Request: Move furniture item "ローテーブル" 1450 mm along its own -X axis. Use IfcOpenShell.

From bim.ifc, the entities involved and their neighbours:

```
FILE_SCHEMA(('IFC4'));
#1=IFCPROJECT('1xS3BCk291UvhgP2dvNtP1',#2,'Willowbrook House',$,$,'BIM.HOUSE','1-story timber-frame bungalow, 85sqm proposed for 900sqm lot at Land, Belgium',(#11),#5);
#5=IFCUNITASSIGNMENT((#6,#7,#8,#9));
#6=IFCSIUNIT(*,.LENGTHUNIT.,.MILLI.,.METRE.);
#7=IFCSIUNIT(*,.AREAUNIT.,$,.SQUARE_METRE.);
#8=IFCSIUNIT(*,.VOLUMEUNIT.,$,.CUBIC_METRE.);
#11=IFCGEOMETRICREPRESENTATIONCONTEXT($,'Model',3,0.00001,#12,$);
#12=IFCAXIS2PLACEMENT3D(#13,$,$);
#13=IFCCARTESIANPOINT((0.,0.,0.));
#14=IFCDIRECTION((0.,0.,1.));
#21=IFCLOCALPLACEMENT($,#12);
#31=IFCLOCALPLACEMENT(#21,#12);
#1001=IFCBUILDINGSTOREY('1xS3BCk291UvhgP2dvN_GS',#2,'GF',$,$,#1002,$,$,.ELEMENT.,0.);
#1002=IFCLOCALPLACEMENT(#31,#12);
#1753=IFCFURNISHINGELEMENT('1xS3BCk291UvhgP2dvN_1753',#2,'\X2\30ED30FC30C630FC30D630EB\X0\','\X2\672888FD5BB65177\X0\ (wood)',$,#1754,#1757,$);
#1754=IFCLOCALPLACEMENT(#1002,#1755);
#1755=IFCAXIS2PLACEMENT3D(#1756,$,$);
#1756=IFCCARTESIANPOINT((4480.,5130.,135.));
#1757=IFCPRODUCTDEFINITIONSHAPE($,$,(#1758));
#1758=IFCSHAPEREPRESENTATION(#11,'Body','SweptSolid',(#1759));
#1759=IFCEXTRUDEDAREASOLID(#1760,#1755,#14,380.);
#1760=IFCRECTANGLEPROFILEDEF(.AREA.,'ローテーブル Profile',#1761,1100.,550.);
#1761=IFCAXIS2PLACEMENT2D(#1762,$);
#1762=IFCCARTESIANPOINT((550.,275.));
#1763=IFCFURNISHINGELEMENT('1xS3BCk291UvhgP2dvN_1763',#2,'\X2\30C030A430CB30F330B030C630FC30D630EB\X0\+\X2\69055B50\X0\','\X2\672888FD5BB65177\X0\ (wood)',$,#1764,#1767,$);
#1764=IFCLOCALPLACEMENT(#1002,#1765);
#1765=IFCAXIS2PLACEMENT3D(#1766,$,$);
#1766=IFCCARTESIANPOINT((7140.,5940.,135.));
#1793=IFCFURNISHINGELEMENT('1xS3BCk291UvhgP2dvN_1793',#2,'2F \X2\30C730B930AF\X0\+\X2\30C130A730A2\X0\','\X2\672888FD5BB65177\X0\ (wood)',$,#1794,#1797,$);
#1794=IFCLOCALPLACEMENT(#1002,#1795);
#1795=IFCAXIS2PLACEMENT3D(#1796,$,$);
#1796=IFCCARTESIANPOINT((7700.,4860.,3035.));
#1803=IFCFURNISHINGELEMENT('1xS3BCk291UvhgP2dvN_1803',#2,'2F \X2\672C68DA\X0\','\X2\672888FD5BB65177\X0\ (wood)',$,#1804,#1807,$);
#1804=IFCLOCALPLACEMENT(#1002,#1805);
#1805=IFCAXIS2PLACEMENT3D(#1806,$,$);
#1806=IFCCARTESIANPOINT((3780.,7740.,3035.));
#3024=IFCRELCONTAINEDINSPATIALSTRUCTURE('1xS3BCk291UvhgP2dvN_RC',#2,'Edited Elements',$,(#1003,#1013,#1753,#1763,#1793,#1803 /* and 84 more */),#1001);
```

```python
import ifcopenshell
import ifcopenshell.api.geometry
import ifcopenshell.util.placement
import ifcopenshell.util.unit

model = ifcopenshell.open("bim.ifc")
unit_scale = ifcopenshell.util.unit.calculate_unit_scale(model)

item = model.by_guid("1xS3BCk291UvhgP2dvN_1753")
matrix = ifcopenshell.util.placement.get_local_placement(item.ObjectPlacement)
matrix[:3, 3] -= matrix[:3, 0] * 1.45 / unit_scale
ifcopenshell.api.geometry.edit_object_placement(model, product=item, matrix=matrix, is_si=False)

print(ifcopenshell.util.placement.get_local_placement(item.ObjectPlacement).round(3) + 0.0)

model.write("bim_updated.ifc")
```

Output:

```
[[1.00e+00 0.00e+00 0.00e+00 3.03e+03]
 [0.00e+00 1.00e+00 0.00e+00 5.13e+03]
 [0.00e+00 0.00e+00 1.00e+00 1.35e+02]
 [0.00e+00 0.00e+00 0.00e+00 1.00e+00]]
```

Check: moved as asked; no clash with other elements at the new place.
